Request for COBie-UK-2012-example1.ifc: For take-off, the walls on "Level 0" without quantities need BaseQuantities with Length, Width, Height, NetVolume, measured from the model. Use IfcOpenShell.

First a look at what the model holds.

```python
import ifcopenshell
import ifcopenshell.util.element
import ifcopenshell.util.unit

model = ifcopenshell.open("COBie-UK-2012-example1.ifc")
print(model.schema)
for unit_type in ("LENGTHUNIT", "AREAUNIT", "VOLUMEUNIT"):
    print(unit_type, ifcopenshell.util.unit.calculate_unit_scale(model, unit_type))
storey = next(s for s in model.by_type("IfcBuildingStorey") if s.Name == "Level 0")
walls = [e for e in ifcopenshell.util.element.get_decomposition(storey) if e.is_a("IfcWall")]
for e in sorted(walls, key=lambda e: e.id()):
    print(e.id(), e.is_a(), e.Name, list(ifcopenshell.util.element.get_psets(e, qtos_only=True)), sep=" | ")
```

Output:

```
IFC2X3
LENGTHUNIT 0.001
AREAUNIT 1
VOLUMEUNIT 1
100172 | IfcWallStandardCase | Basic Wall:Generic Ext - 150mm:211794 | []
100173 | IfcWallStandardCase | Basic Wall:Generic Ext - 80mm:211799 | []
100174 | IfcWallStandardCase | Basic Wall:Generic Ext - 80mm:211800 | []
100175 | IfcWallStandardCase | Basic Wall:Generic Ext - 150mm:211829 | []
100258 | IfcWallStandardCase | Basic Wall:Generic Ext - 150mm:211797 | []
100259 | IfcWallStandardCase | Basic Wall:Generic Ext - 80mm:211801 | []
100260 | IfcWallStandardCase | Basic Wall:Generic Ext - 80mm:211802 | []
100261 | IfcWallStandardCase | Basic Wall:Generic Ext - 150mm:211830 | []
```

```python
import ifcopenshell
import ifcopenshell.api.pset
import ifcopenshell.geom
import ifcopenshell.util.element
import ifcopenshell.util.shape
import ifcopenshell.util.unit

model = ifcopenshell.open("COBie-UK-2012-example1.ifc")
unit_scale = ifcopenshell.util.unit.calculate_unit_scale(model)
volume_scale = ifcopenshell.util.unit.calculate_unit_scale(model, "VOLUMEUNIT")
settings = ifcopenshell.geom.settings()

storey = next(s for s in model.by_type("IfcBuildingStorey") if s.Name == "Level 0")
walls = [e for e in ifcopenshell.util.element.get_decomposition(storey) if e.is_a("IfcWall")]

for e in sorted(walls, key=lambda e: e.id()):
    if ifcopenshell.util.element.get_psets(e, qtos_only=True, should_inherit=False):
        continue
    # Geometry comes back in metres, in the element's own axes.
    shape = ifcopenshell.geom.create_shape(settings, e)
    values = {
        "Length": ifcopenshell.util.shape.get_x(shape.geometry) / unit_scale,
        "Width": ifcopenshell.util.shape.get_y(shape.geometry) / unit_scale,
        "Height": ifcopenshell.util.shape.get_z(shape.geometry) / unit_scale,
        "NetVolume": ifcopenshell.util.shape.get_volume(shape.geometry) / volume_scale,
    }
    qto = ifcopenshell.api.pset.add_qto(model, product=e, name="BaseQuantities")
    ifcopenshell.api.pset.edit_qto(model, qto=qto, properties=values)
    print(e.id(), {k: round(v, 3) for k, v in values.items()})

model.write("COBie-UK-2012-example1_rev.ifc")
```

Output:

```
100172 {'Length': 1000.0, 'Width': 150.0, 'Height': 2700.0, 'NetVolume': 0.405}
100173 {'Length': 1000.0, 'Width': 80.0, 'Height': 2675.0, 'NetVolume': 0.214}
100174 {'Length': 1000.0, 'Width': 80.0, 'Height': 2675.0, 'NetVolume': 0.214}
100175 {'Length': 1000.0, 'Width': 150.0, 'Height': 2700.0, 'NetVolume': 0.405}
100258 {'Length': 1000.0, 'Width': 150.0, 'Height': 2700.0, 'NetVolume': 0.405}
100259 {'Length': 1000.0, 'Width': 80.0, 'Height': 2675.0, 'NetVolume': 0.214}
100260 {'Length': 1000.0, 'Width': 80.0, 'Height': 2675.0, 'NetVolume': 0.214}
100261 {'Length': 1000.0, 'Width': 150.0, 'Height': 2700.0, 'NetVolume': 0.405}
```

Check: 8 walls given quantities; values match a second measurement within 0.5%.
